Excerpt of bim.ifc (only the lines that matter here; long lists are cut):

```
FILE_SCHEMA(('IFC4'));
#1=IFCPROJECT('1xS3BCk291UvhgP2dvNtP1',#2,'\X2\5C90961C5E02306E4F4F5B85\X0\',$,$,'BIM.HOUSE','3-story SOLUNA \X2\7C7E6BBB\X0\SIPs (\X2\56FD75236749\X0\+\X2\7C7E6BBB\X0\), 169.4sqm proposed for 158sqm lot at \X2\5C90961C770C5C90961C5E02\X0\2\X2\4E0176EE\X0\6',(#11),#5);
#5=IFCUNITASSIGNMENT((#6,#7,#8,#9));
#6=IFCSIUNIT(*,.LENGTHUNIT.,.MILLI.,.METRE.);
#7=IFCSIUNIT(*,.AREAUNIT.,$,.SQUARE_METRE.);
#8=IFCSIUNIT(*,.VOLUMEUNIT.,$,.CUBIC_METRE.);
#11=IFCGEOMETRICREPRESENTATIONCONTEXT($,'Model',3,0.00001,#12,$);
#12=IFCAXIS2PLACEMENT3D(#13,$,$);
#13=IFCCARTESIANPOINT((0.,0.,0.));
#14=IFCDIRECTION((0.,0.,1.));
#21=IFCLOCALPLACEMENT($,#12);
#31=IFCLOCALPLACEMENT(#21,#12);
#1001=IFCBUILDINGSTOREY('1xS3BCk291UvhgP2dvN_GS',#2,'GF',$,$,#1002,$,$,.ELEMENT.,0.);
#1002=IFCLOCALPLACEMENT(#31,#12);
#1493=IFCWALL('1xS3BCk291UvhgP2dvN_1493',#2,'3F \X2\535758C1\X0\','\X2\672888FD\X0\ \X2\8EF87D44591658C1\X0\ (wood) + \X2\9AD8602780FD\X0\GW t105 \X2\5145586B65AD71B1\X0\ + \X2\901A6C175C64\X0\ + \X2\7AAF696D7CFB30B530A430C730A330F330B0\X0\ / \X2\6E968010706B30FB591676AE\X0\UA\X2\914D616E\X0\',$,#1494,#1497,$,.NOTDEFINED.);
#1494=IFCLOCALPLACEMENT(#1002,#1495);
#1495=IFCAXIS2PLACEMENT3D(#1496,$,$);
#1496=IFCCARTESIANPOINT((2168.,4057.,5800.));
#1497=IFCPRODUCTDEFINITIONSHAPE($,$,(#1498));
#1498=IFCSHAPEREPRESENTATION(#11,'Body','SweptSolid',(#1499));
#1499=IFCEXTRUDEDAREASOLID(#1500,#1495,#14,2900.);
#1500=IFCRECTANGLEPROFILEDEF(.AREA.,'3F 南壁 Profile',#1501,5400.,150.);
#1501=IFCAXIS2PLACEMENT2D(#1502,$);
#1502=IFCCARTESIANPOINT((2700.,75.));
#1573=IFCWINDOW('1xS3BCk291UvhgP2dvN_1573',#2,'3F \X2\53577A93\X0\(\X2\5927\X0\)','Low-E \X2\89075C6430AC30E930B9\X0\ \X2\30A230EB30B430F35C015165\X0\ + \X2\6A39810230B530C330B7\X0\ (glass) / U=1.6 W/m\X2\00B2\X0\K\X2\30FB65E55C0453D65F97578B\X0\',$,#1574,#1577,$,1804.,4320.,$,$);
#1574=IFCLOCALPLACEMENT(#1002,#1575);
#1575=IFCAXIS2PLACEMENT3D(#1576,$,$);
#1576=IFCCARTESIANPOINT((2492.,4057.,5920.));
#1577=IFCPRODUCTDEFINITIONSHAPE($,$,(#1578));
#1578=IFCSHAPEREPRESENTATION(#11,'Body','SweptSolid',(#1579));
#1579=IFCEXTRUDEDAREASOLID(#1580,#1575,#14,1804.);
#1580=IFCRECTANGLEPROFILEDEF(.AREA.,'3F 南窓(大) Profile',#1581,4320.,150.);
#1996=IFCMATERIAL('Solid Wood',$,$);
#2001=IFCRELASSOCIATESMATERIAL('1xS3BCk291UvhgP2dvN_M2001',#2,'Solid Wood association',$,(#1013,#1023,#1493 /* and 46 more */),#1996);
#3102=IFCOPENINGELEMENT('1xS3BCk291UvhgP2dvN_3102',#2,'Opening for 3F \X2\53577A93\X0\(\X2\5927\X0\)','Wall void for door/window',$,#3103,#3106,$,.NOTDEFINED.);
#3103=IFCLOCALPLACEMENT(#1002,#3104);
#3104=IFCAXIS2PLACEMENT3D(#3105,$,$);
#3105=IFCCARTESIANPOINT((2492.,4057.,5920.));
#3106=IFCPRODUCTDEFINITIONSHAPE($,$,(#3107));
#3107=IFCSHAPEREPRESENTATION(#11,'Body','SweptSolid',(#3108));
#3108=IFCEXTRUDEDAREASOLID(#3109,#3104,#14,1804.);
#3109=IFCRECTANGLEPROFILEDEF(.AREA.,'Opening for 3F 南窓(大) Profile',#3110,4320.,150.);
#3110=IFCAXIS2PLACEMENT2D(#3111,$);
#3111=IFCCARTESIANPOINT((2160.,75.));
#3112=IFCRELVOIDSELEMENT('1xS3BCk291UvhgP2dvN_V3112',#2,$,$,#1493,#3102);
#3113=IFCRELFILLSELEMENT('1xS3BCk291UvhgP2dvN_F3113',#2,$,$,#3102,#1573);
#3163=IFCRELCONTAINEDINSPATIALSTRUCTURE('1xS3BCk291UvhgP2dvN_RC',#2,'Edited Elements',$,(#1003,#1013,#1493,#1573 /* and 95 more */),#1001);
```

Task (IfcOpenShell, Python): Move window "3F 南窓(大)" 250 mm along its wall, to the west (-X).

```python
import ifcopenshell
import ifcopenshell.api.geometry
import ifcopenshell.util.placement
import ifcopenshell.util.unit

model = ifcopenshell.open("bim.ifc")
unit_scale = ifcopenshell.util.unit.calculate_unit_scale(model)

window = model.by_guid("1xS3BCk291UvhgP2dvN_1573")
opening = window.FillsVoids[0].RelatingOpeningElement
wall = opening.VoidsElements[0].RelatingBuildingElement

wall_matrix = ifcopenshell.util.placement.get_local_placement(wall.ObjectPlacement)
shift = wall_matrix[:3, 0] * -0.25 / unit_scale
before = ifcopenshell.util.placement.get_local_placement(window.ObjectPlacement)[:3, 3].copy()

# The window is not placed relative to its opening, so move both.
for product in (opening, window):
    matrix = ifcopenshell.util.placement.get_local_placement(product.ObjectPlacement)
    matrix[:3, 3] += shift
    ifcopenshell.api.geometry.edit_object_placement(model, product=product, matrix=matrix, is_si=False)

after = ifcopenshell.util.placement.get_local_placement(window.ObjectPlacement)[:3, 3]
print("window moved by", (after - before).round(3) + 0.0)

model.write("bim_rev.ifc")
```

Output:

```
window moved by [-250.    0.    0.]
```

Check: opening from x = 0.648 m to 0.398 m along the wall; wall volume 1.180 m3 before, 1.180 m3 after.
